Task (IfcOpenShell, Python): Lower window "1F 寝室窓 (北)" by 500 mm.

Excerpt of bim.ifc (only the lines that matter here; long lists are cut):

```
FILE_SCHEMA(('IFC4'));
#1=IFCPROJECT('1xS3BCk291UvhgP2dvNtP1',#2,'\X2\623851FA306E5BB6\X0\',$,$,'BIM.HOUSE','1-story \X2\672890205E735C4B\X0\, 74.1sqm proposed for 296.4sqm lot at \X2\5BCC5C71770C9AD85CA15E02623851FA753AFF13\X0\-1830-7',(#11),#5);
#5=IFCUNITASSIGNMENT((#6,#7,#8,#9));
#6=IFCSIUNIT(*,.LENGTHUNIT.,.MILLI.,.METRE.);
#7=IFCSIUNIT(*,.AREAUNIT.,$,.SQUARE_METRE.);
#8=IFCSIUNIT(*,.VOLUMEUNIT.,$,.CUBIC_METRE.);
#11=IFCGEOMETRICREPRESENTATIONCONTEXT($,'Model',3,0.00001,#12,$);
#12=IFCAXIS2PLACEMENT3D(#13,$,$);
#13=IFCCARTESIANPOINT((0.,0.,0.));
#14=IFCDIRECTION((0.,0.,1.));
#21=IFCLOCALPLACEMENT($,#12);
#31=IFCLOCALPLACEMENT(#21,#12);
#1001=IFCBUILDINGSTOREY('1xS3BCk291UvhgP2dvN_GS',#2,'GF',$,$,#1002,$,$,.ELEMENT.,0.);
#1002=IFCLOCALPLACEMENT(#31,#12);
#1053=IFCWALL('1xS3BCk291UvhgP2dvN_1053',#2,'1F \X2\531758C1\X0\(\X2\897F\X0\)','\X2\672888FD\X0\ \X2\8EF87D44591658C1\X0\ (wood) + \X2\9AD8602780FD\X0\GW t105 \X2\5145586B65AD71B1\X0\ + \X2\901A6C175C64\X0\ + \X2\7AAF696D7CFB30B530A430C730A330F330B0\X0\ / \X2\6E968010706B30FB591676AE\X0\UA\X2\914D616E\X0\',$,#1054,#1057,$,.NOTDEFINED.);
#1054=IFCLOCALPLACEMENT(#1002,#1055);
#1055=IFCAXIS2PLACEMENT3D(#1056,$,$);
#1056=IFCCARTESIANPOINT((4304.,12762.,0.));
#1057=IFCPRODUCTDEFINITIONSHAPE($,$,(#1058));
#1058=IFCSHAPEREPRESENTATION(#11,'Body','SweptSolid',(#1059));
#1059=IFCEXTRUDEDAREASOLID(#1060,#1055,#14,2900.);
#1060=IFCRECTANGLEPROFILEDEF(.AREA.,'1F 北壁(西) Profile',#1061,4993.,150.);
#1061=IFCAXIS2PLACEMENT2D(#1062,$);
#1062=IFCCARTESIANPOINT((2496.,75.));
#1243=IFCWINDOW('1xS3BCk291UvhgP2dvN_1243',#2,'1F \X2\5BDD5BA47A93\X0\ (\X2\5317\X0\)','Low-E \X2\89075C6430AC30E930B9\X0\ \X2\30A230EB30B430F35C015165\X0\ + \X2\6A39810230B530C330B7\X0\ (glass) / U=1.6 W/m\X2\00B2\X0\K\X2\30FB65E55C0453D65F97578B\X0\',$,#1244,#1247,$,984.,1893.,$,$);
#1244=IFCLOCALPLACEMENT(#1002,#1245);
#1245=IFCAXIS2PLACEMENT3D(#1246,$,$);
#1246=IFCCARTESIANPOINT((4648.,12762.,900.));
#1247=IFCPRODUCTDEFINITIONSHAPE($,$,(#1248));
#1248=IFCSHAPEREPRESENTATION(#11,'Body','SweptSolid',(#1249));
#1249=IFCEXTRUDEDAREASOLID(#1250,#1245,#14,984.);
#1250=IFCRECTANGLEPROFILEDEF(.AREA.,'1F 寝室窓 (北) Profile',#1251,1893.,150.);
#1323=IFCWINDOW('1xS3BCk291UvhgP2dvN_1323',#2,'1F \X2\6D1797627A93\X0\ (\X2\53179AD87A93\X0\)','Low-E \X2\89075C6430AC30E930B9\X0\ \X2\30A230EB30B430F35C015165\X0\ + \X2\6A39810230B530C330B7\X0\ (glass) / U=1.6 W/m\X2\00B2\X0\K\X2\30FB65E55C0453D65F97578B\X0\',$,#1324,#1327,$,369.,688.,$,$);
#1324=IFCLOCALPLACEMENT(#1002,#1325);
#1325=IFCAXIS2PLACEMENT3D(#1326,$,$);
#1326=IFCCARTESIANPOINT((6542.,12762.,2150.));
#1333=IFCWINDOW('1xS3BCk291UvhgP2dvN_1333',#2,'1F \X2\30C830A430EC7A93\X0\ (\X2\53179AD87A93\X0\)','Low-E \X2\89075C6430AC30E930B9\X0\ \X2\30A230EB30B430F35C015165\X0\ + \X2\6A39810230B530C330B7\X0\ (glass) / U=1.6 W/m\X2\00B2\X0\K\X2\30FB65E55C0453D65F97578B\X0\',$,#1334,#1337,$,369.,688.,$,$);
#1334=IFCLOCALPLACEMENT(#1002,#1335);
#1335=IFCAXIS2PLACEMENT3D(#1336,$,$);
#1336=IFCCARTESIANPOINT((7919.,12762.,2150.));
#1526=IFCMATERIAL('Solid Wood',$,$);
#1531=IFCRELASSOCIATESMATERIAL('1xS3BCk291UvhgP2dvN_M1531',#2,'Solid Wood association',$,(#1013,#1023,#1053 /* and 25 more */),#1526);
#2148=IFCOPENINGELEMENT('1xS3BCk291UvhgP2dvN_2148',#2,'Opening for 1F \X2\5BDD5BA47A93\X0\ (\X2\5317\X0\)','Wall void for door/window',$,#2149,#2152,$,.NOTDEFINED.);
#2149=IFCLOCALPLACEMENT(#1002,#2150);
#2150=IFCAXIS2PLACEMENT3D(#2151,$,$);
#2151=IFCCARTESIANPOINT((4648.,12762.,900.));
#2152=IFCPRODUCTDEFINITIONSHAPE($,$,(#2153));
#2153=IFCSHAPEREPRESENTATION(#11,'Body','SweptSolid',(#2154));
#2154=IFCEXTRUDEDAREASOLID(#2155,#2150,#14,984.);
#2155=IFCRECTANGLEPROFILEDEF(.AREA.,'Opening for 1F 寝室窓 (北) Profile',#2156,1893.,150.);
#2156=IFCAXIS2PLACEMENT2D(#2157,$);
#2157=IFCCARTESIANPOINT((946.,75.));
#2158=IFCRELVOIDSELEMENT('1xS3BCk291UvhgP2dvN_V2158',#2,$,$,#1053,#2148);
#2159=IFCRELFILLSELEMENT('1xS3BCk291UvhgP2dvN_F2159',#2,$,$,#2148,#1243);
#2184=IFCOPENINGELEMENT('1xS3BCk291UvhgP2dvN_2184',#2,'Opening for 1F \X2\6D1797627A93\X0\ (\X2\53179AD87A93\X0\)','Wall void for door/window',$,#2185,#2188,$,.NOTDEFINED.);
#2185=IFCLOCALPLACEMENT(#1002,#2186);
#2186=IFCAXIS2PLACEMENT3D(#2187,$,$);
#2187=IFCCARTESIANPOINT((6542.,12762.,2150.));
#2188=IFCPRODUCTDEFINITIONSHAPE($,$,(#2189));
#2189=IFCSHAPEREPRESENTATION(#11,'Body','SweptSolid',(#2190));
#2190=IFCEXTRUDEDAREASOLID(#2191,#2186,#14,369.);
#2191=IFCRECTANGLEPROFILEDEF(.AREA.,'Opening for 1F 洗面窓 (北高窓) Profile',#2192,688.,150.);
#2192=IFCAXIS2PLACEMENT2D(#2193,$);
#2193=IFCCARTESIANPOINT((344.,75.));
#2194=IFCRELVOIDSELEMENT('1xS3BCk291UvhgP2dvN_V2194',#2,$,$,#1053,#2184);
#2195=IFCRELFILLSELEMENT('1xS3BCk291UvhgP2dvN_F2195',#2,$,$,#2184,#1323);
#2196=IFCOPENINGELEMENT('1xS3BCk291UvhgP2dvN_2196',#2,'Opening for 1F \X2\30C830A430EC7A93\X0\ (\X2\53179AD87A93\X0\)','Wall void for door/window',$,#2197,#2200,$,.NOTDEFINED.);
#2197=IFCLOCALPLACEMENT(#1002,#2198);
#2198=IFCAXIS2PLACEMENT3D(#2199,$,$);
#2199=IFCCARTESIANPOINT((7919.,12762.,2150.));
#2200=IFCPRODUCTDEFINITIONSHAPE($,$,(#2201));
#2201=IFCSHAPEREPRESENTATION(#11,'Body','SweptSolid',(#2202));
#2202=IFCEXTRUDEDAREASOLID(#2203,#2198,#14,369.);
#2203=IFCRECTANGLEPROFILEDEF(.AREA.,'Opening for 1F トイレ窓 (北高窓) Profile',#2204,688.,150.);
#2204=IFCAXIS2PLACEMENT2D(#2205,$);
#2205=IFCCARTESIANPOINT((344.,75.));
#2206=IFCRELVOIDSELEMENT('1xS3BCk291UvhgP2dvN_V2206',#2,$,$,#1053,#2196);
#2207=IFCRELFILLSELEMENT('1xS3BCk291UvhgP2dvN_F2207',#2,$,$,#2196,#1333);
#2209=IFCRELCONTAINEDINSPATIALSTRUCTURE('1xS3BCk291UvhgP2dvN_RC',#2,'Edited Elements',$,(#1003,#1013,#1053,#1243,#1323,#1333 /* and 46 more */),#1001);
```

```python
import numpy as np
import ifcopenshell
import ifcopenshell.api.geometry
import ifcopenshell.util.placement
import ifcopenshell.util.unit

model = ifcopenshell.open("bim.ifc")
unit_scale = ifcopenshell.util.unit.calculate_unit_scale(model)

window = model.by_guid("1xS3BCk291UvhgP2dvN_1243")
opening = window.FillsVoids[0].RelatingOpeningElement
dz = -0.5 / unit_scale

shift = np.array([0.0, 0.0, dz])
# The window is not placed relative to its opening, so move both.
for product in (opening, window):
    matrix = ifcopenshell.util.placement.get_local_placement(product.ObjectPlacement)
    matrix[:3, 3] += shift
    ifcopenshell.api.geometry.edit_object_placement(model, product=product, matrix=matrix, is_si=False)

print(f"moved by {dz * unit_scale:+.3f} m")

model.write("bim_updated.ifc")
```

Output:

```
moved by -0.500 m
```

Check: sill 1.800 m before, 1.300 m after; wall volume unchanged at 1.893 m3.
